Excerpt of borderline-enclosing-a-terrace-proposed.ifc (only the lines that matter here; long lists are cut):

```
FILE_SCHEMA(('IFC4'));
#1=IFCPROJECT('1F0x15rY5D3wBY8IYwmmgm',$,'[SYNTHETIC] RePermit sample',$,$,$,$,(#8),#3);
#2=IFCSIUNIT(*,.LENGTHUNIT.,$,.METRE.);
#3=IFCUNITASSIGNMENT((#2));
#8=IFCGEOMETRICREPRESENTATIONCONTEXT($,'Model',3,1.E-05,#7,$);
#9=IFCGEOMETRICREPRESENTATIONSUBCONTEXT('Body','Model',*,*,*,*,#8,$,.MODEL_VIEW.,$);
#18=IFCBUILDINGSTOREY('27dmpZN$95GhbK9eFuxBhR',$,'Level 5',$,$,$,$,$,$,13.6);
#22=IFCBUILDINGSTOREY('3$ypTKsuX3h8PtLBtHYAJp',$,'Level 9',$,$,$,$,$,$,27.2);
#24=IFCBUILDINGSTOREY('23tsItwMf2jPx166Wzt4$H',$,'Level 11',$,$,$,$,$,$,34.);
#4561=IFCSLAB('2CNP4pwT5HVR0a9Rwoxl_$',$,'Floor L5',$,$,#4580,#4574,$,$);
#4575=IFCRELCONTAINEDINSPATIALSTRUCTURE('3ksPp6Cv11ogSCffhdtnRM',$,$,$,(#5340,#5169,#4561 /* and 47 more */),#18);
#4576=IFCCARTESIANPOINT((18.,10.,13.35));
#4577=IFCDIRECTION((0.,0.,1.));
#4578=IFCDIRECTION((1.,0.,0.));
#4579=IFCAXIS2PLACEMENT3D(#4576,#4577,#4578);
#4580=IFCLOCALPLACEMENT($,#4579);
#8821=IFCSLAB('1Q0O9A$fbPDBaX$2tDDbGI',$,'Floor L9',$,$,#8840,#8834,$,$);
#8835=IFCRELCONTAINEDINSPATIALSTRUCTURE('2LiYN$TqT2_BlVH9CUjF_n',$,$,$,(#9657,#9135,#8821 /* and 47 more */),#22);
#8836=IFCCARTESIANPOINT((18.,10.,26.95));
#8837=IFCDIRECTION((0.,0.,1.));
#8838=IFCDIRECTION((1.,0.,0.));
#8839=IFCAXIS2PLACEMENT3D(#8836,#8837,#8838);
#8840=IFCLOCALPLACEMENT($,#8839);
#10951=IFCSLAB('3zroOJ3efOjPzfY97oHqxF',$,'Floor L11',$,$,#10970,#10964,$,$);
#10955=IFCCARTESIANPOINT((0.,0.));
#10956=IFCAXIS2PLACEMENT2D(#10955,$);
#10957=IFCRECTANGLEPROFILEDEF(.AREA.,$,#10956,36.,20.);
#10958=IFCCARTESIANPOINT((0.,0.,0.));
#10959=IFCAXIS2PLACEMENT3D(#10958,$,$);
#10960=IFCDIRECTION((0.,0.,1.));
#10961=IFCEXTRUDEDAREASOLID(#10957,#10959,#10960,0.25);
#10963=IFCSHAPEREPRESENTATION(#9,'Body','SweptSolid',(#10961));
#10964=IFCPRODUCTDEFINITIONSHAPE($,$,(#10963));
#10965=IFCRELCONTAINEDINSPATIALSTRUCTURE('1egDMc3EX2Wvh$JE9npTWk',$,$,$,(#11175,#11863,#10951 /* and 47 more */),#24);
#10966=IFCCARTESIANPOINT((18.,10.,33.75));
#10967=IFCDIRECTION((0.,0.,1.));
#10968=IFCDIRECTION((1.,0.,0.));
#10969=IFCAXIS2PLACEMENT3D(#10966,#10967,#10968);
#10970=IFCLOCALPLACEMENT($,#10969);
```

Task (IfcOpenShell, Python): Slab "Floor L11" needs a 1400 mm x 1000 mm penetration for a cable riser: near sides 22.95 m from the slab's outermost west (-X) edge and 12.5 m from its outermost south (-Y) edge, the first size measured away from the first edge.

```python
import numpy as np
import ifcopenshell
import ifcopenshell.api.feature
import ifcopenshell.api.geometry
import ifcopenshell.api.root
import ifcopenshell.geom
import ifcopenshell.util.placement
import ifcopenshell.util.representation
import ifcopenshell.util.shape
import ifcopenshell.util.unit

model = ifcopenshell.open("borderline-enclosing-a-terrace-proposed.ifc")
unit_scale = ifcopenshell.util.unit.calculate_unit_scale(model)
settings = ifcopenshell.geom.settings()


def volume(element):
    """Net volume in cubic metres, openings subtracted."""
    shape = ifcopenshell.geom.create_shape(settings, element)
    return ifcopenshell.util.shape.get_volume(shape.geometry)


slab = model.by_guid("3zroOJ3efOjPzfY97oHqxF")
before = volume(slab)

# Extent in the slab's own axes, in metres. The edges named are its -X and -Y sides.
slab_shape = ifcopenshell.geom.create_shape(settings, slab)
vertices = ifcopenshell.util.shape.get_vertices(slab_shape.geometry)
x_min, y_min, bottom = vertices.min(axis=0)
top = vertices[:, 2].max()

opening = ifcopenshell.api.root.create_entity(model, ifc_class="IfcOpeningElement", name="Cable riser opening", predefined_type="OPENING")
context = ifcopenshell.util.representation.get_context(model, "Model", "Body", "MODEL_VIEW")
width, depth = 1.4, 1
outline = [(0.0, 0.0), (width, 0.0), (width, depth), (0.0, depth), (0.0, 0.0)]
# Overshoot both faces by 50 mm so the cut is clean.
shape = ifcopenshell.api.geometry.add_slab_representation(
    model, context=context, depth=top - bottom + 0.1, polyline=outline
)
ifcopenshell.api.geometry.assign_representation(model, product=opening, representation=shape)

matrix = ifcopenshell.util.placement.get_local_placement(slab.ObjectPlacement)
matrix[:, 3] = matrix @ np.append(np.array([x_min + 22.95, y_min + 12.5, bottom - 0.05]) / unit_scale, 1.0)
ifcopenshell.api.geometry.edit_object_placement(model, product=opening, matrix=matrix, is_si=False)
ifcopenshell.api.feature.add_feature(model, feature=opening, element=slab)

after = volume(slab)

print(f"slab volume {before:.3f} -> {after:.3f} m3")

model.write("borderline-enclosing-a-terrace-proposed-out.ifc")
```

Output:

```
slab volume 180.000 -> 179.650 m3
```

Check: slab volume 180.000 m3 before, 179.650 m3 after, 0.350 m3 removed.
